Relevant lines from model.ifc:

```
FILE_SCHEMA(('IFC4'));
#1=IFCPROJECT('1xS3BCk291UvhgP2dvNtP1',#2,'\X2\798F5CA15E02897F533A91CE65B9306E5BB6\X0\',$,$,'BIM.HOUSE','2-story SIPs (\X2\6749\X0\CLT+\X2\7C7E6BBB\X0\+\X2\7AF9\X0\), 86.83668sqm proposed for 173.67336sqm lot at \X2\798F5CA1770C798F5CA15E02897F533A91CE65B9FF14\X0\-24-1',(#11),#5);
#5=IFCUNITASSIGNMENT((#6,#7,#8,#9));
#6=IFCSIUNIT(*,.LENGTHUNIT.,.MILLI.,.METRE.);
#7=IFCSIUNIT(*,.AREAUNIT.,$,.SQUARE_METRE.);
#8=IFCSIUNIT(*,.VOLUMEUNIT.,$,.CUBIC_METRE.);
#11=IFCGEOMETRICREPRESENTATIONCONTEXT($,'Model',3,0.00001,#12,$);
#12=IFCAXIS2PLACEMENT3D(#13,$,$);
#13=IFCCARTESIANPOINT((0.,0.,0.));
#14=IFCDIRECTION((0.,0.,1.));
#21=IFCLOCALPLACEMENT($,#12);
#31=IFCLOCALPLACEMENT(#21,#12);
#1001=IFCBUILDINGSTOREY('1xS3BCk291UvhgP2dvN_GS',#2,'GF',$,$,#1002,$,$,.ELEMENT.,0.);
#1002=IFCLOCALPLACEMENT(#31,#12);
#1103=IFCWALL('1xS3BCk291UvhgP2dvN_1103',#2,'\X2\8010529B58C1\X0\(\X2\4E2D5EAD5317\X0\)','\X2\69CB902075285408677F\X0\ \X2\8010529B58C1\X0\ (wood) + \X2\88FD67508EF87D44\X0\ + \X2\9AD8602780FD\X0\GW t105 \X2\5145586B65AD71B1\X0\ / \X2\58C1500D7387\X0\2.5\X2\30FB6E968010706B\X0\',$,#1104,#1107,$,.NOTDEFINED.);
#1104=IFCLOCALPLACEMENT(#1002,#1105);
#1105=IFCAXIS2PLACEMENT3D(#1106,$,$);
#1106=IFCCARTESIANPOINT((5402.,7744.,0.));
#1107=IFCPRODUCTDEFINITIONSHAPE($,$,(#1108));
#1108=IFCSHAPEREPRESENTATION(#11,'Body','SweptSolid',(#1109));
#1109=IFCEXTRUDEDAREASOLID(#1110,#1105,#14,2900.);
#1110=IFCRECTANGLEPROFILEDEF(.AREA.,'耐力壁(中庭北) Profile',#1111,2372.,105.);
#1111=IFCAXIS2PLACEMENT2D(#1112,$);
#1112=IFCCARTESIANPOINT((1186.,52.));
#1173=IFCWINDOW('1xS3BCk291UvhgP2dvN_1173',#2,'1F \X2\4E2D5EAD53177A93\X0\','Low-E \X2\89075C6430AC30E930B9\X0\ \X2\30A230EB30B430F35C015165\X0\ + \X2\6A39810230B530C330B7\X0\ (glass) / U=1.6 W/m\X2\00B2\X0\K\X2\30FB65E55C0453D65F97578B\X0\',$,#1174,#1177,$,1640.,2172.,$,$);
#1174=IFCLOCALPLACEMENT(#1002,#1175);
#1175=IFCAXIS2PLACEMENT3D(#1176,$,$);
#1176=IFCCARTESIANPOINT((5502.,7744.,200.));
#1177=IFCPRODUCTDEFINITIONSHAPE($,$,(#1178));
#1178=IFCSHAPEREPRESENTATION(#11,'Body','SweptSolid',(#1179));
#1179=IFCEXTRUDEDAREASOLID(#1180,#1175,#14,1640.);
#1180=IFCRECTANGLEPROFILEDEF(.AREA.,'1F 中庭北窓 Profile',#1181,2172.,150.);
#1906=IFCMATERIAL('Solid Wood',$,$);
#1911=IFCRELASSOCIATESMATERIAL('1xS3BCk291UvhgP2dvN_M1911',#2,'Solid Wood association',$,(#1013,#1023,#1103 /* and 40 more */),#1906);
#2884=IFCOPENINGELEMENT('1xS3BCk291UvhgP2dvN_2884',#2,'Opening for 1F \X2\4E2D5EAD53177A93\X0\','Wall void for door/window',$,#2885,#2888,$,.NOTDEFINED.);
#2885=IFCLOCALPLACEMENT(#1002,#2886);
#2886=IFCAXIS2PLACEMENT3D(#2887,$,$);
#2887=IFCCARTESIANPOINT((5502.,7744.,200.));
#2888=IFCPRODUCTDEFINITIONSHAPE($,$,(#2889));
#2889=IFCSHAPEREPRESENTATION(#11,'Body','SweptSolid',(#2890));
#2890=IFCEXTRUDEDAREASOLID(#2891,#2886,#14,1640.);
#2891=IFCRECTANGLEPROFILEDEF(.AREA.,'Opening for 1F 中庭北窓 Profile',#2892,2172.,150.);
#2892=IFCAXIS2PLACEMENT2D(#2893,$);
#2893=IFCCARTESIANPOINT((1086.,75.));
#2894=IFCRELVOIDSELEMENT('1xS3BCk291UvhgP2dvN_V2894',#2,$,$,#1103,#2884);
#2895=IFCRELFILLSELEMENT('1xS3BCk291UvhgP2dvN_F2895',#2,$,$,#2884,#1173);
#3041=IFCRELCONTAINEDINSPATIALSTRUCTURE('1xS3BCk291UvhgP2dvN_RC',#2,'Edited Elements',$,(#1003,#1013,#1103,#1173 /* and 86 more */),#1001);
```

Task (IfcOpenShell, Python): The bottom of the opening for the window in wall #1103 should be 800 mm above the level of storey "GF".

```python
import numpy as np
import ifcopenshell
import ifcopenshell.api.geometry
import ifcopenshell.geom
import ifcopenshell.util.element
import ifcopenshell.util.placement
import ifcopenshell.util.shape
import ifcopenshell.util.unit

model = ifcopenshell.open("model.ifc")
unit_scale = ifcopenshell.util.unit.calculate_unit_scale(model)

window = model.by_guid("1xS3BCk291UvhgP2dvN_1173")
opening = window.FillsVoids[0].RelatingOpeningElement
storey = ifcopenshell.util.element.get_container(window, ifc_class="IfcBuildingStorey")
level = ifcopenshell.util.placement.get_local_placement(storey.ObjectPlacement)[2, 3]

# The opening's origin need not be at the sill, so measure its lowest point.
shape = ifcopenshell.geom.create_shape(ifcopenshell.geom.settings(), opening)
bottom = ifcopenshell.util.shape.get_shape_bottom_elevation(shape, shape.geometry) / unit_scale
dz = level + 800.0 - bottom

shift = np.array([0.0, 0.0, dz])
# The window is not placed relative to its opening, so move both.
for product in (opening, window):
    matrix = ifcopenshell.util.placement.get_local_placement(product.ObjectPlacement)
    matrix[:3, 3] += shift
    ifcopenshell.api.geometry.edit_object_placement(model, product=product, matrix=matrix, is_si=False)

print(f"moved by {dz * unit_scale:+.3f} m")

model.write("model-out.ifc")
```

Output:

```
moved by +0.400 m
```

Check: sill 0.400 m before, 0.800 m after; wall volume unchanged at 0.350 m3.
